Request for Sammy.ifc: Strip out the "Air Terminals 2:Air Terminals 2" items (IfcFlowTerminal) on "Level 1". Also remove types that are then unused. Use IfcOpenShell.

First a look at what the model holds.

```python
import ifcopenshell
import ifcopenshell.util.element

model = ifcopenshell.open("Sammy.ifc")
print(model.schema)
storey = next(s for s in model.by_type("IfcBuildingStorey") if s.Name == "Level 1")
terminals = [e for e in ifcopenshell.util.element.get_decomposition(storey) if e.is_a("IfcFlowTerminal")]
seen = {}
for e in terminals:
    element_type = ifcopenshell.util.element.get_type(e)
    name = element_type.Name if element_type not in (None, e) else None
    seen[name] = seen.get(name, 0) + 1
for name, count in sorted(seen.items(), key=str):
    print(count, "x", name)
```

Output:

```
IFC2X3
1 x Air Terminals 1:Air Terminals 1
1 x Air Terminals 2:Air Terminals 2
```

```python
import ifcopenshell
import ifcopenshell.api.root
import ifcopenshell.util.element

model = ifcopenshell.open("Sammy.ifc")

storey = next(s for s in model.by_type("IfcBuildingStorey") if s.Name == "Level 1")
terminals = [e for e in ifcopenshell.util.element.get_decomposition(storey) if e.is_a("IfcFlowTerminal")]
targets = [e for e in terminals if (t := ifcopenshell.util.element.get_type(e)) not in (None, e) and t.Name == "Air Terminals 2:Air Terminals 2"]
types = {ifcopenshell.util.element.get_type(e) for e in targets} - {None, *targets}

for e in targets:
    ifcopenshell.api.root.remove_product(model, product=e)
print(len(targets), "removed")

unused = [t for t in types if not ifcopenshell.util.element.get_types(t)]
for t in unused:
    ifcopenshell.api.root.remove_product(model, product=t)
print(len(unused), "unused types removed")

model.write("Sammy_edited.ifc")
```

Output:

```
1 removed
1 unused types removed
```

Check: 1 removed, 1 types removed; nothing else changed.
